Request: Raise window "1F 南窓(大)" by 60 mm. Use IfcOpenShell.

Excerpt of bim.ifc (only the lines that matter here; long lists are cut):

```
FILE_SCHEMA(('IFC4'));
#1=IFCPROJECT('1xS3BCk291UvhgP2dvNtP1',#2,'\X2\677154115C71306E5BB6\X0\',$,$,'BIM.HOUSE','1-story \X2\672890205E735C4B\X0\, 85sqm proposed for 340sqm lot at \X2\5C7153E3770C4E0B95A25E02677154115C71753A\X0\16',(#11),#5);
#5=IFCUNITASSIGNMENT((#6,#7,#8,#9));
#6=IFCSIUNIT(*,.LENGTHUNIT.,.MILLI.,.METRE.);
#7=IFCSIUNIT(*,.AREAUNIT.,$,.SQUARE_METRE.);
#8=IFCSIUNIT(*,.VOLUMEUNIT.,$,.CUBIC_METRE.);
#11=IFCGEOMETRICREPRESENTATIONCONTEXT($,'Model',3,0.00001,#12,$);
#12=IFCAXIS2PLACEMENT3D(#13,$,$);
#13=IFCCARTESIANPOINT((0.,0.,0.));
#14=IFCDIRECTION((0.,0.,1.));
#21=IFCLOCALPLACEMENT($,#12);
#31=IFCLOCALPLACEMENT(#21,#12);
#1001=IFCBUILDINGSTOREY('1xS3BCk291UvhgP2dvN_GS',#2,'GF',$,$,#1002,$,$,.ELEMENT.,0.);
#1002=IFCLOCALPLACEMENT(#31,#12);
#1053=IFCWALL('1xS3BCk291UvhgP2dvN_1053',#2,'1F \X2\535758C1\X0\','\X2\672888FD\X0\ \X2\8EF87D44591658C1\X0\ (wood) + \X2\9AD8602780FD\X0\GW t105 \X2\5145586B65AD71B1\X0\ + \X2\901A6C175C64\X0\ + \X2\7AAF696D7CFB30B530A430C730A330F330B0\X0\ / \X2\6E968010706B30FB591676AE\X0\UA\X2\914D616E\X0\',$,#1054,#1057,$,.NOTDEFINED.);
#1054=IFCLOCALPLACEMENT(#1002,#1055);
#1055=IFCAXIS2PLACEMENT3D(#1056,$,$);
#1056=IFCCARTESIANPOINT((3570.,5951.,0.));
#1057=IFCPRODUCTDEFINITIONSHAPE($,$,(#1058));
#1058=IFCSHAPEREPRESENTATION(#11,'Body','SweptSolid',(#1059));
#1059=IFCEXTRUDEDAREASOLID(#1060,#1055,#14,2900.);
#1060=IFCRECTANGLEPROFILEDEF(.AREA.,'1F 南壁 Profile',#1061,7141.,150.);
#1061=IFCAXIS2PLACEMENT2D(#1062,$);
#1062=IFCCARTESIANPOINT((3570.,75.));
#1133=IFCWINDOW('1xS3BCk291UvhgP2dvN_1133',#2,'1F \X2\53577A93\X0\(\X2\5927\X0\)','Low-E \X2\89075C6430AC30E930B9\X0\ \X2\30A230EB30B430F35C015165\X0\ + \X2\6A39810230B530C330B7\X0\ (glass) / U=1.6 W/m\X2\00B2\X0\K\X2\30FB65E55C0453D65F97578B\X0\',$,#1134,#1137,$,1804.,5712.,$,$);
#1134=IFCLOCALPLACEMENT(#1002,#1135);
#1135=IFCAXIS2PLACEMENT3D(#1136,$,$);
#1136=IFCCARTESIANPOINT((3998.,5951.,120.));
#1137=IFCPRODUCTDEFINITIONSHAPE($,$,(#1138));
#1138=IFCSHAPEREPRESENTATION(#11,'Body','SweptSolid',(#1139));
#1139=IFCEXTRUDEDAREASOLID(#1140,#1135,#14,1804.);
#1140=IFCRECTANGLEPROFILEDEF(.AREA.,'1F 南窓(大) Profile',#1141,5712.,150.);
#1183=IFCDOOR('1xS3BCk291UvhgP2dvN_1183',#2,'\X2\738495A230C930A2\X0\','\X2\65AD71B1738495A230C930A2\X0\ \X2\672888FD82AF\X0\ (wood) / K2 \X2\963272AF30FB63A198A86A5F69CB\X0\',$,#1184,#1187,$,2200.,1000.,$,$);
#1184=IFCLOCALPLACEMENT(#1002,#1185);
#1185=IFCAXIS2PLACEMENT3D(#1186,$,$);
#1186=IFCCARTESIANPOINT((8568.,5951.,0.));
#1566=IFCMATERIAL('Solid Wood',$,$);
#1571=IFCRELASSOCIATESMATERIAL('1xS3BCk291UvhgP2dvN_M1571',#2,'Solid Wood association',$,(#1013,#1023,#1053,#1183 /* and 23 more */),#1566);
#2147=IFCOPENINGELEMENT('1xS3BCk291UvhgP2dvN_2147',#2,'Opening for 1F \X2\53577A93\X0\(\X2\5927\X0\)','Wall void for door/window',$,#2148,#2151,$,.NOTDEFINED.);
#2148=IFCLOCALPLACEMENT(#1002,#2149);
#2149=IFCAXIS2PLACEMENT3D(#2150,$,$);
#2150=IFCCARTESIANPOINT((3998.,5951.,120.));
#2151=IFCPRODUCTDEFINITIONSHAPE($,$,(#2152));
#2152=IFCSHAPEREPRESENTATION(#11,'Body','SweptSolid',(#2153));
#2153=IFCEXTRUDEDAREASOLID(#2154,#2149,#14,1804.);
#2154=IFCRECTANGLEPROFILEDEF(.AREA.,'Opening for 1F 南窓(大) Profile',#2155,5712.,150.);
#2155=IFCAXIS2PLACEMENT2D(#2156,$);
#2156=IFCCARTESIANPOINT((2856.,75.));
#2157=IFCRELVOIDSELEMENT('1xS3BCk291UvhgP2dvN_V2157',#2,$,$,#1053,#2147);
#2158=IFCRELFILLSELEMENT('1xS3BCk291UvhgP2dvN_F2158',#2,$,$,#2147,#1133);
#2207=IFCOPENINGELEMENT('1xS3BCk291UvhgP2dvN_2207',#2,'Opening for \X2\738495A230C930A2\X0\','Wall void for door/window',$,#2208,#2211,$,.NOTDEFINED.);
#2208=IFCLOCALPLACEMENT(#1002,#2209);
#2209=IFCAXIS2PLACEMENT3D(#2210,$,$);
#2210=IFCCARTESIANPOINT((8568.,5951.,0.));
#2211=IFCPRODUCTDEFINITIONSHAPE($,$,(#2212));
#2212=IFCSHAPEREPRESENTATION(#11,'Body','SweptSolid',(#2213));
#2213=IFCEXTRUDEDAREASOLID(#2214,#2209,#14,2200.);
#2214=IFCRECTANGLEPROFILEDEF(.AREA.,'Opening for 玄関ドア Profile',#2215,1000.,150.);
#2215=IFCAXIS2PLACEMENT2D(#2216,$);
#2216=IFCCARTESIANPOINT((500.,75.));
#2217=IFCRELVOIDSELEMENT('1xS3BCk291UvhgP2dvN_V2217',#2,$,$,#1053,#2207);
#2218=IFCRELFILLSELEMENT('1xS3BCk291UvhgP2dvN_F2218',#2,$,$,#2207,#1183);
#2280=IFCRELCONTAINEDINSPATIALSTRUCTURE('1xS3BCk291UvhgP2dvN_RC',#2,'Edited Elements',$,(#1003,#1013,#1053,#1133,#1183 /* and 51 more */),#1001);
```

```python
import numpy as np
import ifcopenshell
import ifcopenshell.api.geometry
import ifcopenshell.util.placement
import ifcopenshell.util.unit

model = ifcopenshell.open("bim.ifc")
unit_scale = ifcopenshell.util.unit.calculate_unit_scale(model)

window = model.by_id(1133)
opening = window.FillsVoids[0].RelatingOpeningElement
dz = 0.06 / unit_scale

shift = np.array([0.0, 0.0, dz])
# The window is not placed relative to its opening, so move both.
for product in (opening, window):
    matrix = ifcopenshell.util.placement.get_local_placement(product.ObjectPlacement)
    matrix[:3, 3] += shift
    ifcopenshell.api.geometry.edit_object_placement(model, product=product, matrix=matrix, is_si=False)

print(f"moved by {dz * unit_scale:+.3f} m")

model.write("bim_v2.ifc")
```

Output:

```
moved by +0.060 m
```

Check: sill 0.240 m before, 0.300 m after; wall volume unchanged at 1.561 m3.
